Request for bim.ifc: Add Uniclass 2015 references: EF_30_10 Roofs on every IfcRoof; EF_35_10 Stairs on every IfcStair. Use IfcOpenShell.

First a look at what the model holds.

```python
import ifcopenshell

model = ifcopenshell.open("bim.ifc")
print(model.schema)
print("classifications:", [c.Name for c in model.by_type("IfcClassification")])
for ifc_class in ("IfcDoor", "IfcRoof", "IfcStair", "IfcWall", "IfcWindow"):
    print(ifc_class, len(model.by_type(ifc_class)))
```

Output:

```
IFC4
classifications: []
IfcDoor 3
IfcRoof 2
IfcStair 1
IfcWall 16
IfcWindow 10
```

```python
import ifcopenshell
import ifcopenshell.api.classification

model = ifcopenshell.open("bim.ifc")

system = ifcopenshell.api.classification.add_classification(model, classification="Uniclass 2015")

codes = {
    "IfcRoof": ("EF_30_10", "Roofs"),
    "IfcStair": ("EF_35_10", "Stairs"),
}
for ifc_class, (code, name) in codes.items():
    products = model.by_type(ifc_class)
    ifcopenshell.api.classification.add_reference(
        model, products=products, classification=system, identification=code, name=name
    )
    print(code, len(products))

model.write("bim_updated.ifc")
```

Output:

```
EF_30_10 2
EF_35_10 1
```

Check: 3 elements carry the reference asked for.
